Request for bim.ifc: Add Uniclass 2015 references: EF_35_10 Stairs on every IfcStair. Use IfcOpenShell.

First a look at what the model holds.

```python
import ifcopenshell

model = ifcopenshell.open("bim.ifc")
print(model.schema)
print("classifications:", [c.Name for c in model.by_type("IfcClassification")])
for ifc_class in ("IfcDoor", "IfcRoof", "IfcStair", "IfcWall", "IfcWindow"):
    print(ifc_class, len(model.by_type(ifc_class)))
```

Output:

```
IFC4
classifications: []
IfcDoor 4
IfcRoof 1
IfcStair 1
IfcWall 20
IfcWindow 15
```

```python
import ifcopenshell
import ifcopenshell.api.classification

model = ifcopenshell.open("bim.ifc")

system = ifcopenshell.api.classification.add_classification(model, classification="Uniclass 2015")

codes = {
    "IfcStair": ("EF_35_10", "Stairs"),
}
for ifc_class, (code, name) in codes.items():
    products = model.by_type(ifc_class)
    ifcopenshell.api.classification.add_reference(
        model, products=products, classification=system, identification=code, name=name
    )
    print(code, len(products))

model.write("bim_v2.ifc")
```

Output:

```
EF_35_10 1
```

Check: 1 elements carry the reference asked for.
